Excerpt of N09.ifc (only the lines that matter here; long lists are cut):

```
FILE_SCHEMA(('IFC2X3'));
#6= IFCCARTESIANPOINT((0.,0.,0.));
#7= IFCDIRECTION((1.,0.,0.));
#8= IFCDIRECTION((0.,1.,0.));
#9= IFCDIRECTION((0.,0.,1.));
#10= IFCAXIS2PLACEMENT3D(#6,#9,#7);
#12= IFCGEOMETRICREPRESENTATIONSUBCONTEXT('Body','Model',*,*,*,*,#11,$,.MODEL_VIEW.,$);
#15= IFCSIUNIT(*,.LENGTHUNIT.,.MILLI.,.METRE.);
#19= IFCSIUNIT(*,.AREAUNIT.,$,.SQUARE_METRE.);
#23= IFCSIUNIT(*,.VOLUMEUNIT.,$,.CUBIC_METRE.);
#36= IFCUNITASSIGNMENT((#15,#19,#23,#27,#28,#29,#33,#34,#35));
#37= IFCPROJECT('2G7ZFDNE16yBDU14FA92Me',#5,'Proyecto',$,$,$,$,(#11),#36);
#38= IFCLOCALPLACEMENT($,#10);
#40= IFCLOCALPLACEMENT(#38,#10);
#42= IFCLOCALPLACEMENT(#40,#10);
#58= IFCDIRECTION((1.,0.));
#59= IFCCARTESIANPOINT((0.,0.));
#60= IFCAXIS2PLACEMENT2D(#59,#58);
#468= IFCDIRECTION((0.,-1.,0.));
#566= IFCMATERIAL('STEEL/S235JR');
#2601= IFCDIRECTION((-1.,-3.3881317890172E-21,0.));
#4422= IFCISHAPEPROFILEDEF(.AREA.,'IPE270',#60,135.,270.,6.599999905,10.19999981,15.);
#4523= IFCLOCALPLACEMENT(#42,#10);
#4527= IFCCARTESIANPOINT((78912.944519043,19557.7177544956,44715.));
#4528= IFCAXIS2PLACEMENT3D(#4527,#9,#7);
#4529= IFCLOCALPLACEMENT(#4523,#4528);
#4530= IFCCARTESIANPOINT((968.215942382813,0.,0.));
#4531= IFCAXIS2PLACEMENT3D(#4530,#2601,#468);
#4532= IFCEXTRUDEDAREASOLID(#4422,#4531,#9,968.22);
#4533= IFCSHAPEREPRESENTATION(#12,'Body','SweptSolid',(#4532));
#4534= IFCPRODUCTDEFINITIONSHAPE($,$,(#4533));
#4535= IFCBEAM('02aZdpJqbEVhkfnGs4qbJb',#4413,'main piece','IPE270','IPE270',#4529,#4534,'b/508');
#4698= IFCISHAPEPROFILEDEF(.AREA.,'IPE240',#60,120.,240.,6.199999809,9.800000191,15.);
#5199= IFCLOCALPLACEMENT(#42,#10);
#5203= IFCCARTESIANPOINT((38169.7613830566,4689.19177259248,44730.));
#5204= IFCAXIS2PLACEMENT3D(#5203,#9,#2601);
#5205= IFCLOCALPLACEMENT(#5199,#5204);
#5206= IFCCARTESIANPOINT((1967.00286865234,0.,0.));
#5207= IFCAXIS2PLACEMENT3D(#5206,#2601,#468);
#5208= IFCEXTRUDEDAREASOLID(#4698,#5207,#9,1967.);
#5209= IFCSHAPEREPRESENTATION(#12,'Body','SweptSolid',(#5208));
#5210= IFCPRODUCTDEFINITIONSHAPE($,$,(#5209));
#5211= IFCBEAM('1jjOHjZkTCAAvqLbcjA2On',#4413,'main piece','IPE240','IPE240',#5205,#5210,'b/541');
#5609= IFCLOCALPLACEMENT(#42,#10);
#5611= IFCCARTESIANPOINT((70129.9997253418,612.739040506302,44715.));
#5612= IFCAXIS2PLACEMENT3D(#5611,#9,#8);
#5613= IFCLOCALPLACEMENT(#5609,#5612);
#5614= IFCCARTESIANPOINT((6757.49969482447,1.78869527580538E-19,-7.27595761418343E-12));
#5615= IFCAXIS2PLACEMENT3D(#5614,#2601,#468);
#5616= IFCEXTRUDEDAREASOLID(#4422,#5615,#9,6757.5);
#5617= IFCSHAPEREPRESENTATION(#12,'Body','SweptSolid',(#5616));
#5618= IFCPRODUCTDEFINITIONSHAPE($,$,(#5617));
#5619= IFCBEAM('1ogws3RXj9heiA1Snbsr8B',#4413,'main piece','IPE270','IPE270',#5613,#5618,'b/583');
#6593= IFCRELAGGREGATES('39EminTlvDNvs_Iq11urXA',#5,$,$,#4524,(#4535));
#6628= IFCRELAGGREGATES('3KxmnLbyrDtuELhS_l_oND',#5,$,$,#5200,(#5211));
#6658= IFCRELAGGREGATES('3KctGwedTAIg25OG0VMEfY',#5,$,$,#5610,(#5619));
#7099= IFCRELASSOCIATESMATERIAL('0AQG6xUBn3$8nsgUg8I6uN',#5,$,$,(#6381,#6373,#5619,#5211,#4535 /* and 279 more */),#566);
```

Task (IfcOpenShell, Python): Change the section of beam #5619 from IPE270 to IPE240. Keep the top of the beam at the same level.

```python
import ifcopenshell
import ifcopenshell.util.element
import ifcopenshell.util.representation

model = ifcopenshell.open("N09.ifc")

member = model.by_id(5619)
source = next(p for p in model.by_type("IfcIShapeProfileDef") if p.ProfileName == "IPE240")

body = ifcopenshell.util.representation.get_representation(member, "Model", "Body")
solid = body.Items[0]
old_profile = solid.SweptArea

# Copy the section's sizes but keep this member's own profile position.
profile = ifcopenshell.util.element.copy(model, source)
# Profiles are centred, so shift by half the change in depth to hold the top.
shift = (old_profile.OverallDepth - profile.OverallDepth) / 2
x, y = old_profile.Position.Location.Coordinates
up = (0.0, 1.0)  # upwards, in the solid's own plane
location = model.createIfcCartesianPoint((x + up[0] * shift, y + up[1] * shift))
profile.Position = model.createIfcAxis2Placement2D(location, old_profile.Position.RefDirection)
solid.SweptArea = profile
if not model.get_total_inverses(old_profile):
    ifcopenshell.util.element.remove_deep2(model, old_profile)
member.Description = member.Description.replace("IPE270", "IPE240")
member.ObjectType = member.ObjectType.replace("IPE270", "IPE240")

print(solid.SweptArea)

model.write("N09_rev.ifc")
```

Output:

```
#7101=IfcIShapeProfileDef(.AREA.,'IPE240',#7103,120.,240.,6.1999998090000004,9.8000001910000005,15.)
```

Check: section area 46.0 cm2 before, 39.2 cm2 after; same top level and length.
